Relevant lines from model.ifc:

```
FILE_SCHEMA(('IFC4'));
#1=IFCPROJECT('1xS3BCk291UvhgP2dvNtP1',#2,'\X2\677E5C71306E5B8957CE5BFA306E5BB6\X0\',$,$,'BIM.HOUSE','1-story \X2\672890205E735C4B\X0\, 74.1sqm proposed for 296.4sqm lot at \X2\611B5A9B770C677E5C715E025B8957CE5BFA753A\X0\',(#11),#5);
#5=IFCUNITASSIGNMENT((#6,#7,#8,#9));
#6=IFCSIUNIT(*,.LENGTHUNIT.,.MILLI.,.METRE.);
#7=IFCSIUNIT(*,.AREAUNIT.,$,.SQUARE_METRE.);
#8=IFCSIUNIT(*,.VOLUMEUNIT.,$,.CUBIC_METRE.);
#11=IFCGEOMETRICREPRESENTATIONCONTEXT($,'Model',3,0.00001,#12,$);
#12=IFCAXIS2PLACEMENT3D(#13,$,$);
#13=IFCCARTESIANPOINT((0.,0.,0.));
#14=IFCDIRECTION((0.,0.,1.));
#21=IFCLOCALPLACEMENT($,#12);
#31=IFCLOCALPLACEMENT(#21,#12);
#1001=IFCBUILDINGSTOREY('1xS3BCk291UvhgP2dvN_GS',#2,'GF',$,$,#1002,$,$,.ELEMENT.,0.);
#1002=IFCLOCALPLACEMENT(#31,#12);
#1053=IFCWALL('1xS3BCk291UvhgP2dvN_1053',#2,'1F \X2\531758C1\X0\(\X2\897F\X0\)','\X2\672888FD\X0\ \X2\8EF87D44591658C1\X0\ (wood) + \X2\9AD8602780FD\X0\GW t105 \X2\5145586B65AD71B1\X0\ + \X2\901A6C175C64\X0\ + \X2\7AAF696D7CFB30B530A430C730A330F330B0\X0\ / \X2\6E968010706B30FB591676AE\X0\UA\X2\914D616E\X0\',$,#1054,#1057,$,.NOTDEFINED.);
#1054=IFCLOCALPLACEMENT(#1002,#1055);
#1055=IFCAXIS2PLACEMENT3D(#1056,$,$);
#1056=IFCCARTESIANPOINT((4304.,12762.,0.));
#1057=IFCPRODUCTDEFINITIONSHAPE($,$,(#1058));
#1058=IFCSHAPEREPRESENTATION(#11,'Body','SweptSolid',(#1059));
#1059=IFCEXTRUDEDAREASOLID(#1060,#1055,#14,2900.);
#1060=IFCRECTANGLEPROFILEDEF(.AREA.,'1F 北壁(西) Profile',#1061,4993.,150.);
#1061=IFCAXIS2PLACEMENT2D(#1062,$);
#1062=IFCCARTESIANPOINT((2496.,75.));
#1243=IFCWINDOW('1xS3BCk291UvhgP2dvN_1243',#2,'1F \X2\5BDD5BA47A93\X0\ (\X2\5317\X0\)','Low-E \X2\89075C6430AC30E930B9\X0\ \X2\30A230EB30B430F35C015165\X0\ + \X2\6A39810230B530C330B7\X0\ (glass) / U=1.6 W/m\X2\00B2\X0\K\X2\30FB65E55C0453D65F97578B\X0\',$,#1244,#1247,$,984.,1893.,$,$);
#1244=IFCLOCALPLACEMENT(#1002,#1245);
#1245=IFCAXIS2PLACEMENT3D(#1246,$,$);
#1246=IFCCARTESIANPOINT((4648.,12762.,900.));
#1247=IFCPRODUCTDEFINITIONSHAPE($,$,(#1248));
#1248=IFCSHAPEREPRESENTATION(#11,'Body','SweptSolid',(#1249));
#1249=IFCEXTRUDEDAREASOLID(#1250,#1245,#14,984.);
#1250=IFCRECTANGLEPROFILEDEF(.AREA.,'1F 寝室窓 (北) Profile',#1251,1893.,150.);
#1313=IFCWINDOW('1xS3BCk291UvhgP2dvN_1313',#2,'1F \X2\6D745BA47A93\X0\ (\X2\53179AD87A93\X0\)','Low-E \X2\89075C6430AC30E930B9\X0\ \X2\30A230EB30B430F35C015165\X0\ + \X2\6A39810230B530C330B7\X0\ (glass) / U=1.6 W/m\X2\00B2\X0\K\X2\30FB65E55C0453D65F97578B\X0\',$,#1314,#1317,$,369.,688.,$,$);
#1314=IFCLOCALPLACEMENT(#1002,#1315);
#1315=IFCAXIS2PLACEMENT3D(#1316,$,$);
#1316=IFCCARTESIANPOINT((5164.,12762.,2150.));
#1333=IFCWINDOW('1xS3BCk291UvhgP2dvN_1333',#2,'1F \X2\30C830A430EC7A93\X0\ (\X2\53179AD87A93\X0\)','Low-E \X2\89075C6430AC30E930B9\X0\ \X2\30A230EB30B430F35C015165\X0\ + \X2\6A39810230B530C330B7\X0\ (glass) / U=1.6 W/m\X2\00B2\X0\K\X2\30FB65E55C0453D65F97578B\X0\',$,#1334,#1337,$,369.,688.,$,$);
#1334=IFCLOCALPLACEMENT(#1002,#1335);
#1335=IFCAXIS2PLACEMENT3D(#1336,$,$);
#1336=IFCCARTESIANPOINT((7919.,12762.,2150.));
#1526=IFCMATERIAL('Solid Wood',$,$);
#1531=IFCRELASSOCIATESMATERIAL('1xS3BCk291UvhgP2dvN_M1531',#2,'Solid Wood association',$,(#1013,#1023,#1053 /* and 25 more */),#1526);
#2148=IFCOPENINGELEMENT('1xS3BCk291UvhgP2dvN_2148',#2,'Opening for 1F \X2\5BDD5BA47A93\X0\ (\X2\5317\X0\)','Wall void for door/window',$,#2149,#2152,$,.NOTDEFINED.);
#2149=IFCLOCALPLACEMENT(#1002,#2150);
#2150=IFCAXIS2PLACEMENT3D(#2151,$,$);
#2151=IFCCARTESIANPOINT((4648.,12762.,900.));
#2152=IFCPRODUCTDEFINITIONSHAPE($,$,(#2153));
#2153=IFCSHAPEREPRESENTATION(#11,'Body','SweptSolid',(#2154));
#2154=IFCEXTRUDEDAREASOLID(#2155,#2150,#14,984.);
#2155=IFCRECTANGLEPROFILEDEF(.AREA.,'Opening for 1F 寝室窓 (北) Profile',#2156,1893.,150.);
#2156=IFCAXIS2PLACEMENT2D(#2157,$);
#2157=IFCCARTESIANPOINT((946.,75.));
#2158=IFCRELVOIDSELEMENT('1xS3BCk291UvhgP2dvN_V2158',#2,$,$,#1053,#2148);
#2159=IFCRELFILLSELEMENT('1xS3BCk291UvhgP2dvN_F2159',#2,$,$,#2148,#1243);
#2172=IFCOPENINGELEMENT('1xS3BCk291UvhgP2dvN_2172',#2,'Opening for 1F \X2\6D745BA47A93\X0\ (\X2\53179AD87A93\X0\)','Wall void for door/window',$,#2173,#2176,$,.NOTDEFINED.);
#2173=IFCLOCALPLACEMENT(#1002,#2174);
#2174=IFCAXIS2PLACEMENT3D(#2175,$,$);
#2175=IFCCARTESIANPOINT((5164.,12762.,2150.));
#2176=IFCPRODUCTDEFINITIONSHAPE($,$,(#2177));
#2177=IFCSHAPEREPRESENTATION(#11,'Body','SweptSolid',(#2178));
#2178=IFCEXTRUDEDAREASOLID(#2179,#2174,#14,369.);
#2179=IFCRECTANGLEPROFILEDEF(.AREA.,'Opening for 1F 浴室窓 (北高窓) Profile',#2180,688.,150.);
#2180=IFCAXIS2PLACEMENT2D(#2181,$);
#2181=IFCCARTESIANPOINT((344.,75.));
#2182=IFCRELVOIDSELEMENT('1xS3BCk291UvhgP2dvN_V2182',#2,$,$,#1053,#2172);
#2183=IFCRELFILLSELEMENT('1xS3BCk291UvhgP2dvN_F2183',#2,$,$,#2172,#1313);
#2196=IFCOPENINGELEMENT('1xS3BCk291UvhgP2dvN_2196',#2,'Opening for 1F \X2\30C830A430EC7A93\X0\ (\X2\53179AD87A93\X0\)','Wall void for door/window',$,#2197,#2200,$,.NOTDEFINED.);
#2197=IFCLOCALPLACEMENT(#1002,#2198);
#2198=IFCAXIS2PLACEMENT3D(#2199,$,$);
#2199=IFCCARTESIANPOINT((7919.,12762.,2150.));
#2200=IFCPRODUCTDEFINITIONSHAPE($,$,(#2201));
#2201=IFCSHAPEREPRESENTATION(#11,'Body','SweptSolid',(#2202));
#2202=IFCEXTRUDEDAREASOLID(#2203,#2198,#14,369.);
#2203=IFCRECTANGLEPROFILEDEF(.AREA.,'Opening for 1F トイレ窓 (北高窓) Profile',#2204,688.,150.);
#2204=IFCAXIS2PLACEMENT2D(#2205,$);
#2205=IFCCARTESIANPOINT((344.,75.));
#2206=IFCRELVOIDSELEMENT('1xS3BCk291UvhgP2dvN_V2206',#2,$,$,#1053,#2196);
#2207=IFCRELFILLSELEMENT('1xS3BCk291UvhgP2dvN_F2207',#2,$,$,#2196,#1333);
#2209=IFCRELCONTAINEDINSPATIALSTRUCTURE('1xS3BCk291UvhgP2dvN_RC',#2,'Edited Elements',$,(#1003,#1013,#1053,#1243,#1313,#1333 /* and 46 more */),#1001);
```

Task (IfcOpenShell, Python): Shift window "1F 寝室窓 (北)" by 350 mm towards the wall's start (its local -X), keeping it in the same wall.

```python
import ifcopenshell
import ifcopenshell.api.geometry
import ifcopenshell.util.placement
import ifcopenshell.util.unit

model = ifcopenshell.open("model.ifc")
unit_scale = ifcopenshell.util.unit.calculate_unit_scale(model)

window = model.by_id(1243)
opening = window.FillsVoids[0].RelatingOpeningElement
wall = opening.VoidsElements[0].RelatingBuildingElement

wall_matrix = ifcopenshell.util.placement.get_local_placement(wall.ObjectPlacement)
shift = wall_matrix[:3, 0] * -0.35 / unit_scale
before = ifcopenshell.util.placement.get_local_placement(window.ObjectPlacement)[:3, 3].copy()

# The window is not placed relative to its opening, so move both.
for product in (opening, window):
    matrix = ifcopenshell.util.placement.get_local_placement(product.ObjectPlacement)
    matrix[:3, 3] += shift
    ifcopenshell.api.geometry.edit_object_placement(model, product=product, matrix=matrix, is_si=False)

after = ifcopenshell.util.placement.get_local_placement(window.ObjectPlacement)[:3, 3]
print("window moved by", (after - before).round(3) + 0.0)

model.write("model_v2.ifc")
```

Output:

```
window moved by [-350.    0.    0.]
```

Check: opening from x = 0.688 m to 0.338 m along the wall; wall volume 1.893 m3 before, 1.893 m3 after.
